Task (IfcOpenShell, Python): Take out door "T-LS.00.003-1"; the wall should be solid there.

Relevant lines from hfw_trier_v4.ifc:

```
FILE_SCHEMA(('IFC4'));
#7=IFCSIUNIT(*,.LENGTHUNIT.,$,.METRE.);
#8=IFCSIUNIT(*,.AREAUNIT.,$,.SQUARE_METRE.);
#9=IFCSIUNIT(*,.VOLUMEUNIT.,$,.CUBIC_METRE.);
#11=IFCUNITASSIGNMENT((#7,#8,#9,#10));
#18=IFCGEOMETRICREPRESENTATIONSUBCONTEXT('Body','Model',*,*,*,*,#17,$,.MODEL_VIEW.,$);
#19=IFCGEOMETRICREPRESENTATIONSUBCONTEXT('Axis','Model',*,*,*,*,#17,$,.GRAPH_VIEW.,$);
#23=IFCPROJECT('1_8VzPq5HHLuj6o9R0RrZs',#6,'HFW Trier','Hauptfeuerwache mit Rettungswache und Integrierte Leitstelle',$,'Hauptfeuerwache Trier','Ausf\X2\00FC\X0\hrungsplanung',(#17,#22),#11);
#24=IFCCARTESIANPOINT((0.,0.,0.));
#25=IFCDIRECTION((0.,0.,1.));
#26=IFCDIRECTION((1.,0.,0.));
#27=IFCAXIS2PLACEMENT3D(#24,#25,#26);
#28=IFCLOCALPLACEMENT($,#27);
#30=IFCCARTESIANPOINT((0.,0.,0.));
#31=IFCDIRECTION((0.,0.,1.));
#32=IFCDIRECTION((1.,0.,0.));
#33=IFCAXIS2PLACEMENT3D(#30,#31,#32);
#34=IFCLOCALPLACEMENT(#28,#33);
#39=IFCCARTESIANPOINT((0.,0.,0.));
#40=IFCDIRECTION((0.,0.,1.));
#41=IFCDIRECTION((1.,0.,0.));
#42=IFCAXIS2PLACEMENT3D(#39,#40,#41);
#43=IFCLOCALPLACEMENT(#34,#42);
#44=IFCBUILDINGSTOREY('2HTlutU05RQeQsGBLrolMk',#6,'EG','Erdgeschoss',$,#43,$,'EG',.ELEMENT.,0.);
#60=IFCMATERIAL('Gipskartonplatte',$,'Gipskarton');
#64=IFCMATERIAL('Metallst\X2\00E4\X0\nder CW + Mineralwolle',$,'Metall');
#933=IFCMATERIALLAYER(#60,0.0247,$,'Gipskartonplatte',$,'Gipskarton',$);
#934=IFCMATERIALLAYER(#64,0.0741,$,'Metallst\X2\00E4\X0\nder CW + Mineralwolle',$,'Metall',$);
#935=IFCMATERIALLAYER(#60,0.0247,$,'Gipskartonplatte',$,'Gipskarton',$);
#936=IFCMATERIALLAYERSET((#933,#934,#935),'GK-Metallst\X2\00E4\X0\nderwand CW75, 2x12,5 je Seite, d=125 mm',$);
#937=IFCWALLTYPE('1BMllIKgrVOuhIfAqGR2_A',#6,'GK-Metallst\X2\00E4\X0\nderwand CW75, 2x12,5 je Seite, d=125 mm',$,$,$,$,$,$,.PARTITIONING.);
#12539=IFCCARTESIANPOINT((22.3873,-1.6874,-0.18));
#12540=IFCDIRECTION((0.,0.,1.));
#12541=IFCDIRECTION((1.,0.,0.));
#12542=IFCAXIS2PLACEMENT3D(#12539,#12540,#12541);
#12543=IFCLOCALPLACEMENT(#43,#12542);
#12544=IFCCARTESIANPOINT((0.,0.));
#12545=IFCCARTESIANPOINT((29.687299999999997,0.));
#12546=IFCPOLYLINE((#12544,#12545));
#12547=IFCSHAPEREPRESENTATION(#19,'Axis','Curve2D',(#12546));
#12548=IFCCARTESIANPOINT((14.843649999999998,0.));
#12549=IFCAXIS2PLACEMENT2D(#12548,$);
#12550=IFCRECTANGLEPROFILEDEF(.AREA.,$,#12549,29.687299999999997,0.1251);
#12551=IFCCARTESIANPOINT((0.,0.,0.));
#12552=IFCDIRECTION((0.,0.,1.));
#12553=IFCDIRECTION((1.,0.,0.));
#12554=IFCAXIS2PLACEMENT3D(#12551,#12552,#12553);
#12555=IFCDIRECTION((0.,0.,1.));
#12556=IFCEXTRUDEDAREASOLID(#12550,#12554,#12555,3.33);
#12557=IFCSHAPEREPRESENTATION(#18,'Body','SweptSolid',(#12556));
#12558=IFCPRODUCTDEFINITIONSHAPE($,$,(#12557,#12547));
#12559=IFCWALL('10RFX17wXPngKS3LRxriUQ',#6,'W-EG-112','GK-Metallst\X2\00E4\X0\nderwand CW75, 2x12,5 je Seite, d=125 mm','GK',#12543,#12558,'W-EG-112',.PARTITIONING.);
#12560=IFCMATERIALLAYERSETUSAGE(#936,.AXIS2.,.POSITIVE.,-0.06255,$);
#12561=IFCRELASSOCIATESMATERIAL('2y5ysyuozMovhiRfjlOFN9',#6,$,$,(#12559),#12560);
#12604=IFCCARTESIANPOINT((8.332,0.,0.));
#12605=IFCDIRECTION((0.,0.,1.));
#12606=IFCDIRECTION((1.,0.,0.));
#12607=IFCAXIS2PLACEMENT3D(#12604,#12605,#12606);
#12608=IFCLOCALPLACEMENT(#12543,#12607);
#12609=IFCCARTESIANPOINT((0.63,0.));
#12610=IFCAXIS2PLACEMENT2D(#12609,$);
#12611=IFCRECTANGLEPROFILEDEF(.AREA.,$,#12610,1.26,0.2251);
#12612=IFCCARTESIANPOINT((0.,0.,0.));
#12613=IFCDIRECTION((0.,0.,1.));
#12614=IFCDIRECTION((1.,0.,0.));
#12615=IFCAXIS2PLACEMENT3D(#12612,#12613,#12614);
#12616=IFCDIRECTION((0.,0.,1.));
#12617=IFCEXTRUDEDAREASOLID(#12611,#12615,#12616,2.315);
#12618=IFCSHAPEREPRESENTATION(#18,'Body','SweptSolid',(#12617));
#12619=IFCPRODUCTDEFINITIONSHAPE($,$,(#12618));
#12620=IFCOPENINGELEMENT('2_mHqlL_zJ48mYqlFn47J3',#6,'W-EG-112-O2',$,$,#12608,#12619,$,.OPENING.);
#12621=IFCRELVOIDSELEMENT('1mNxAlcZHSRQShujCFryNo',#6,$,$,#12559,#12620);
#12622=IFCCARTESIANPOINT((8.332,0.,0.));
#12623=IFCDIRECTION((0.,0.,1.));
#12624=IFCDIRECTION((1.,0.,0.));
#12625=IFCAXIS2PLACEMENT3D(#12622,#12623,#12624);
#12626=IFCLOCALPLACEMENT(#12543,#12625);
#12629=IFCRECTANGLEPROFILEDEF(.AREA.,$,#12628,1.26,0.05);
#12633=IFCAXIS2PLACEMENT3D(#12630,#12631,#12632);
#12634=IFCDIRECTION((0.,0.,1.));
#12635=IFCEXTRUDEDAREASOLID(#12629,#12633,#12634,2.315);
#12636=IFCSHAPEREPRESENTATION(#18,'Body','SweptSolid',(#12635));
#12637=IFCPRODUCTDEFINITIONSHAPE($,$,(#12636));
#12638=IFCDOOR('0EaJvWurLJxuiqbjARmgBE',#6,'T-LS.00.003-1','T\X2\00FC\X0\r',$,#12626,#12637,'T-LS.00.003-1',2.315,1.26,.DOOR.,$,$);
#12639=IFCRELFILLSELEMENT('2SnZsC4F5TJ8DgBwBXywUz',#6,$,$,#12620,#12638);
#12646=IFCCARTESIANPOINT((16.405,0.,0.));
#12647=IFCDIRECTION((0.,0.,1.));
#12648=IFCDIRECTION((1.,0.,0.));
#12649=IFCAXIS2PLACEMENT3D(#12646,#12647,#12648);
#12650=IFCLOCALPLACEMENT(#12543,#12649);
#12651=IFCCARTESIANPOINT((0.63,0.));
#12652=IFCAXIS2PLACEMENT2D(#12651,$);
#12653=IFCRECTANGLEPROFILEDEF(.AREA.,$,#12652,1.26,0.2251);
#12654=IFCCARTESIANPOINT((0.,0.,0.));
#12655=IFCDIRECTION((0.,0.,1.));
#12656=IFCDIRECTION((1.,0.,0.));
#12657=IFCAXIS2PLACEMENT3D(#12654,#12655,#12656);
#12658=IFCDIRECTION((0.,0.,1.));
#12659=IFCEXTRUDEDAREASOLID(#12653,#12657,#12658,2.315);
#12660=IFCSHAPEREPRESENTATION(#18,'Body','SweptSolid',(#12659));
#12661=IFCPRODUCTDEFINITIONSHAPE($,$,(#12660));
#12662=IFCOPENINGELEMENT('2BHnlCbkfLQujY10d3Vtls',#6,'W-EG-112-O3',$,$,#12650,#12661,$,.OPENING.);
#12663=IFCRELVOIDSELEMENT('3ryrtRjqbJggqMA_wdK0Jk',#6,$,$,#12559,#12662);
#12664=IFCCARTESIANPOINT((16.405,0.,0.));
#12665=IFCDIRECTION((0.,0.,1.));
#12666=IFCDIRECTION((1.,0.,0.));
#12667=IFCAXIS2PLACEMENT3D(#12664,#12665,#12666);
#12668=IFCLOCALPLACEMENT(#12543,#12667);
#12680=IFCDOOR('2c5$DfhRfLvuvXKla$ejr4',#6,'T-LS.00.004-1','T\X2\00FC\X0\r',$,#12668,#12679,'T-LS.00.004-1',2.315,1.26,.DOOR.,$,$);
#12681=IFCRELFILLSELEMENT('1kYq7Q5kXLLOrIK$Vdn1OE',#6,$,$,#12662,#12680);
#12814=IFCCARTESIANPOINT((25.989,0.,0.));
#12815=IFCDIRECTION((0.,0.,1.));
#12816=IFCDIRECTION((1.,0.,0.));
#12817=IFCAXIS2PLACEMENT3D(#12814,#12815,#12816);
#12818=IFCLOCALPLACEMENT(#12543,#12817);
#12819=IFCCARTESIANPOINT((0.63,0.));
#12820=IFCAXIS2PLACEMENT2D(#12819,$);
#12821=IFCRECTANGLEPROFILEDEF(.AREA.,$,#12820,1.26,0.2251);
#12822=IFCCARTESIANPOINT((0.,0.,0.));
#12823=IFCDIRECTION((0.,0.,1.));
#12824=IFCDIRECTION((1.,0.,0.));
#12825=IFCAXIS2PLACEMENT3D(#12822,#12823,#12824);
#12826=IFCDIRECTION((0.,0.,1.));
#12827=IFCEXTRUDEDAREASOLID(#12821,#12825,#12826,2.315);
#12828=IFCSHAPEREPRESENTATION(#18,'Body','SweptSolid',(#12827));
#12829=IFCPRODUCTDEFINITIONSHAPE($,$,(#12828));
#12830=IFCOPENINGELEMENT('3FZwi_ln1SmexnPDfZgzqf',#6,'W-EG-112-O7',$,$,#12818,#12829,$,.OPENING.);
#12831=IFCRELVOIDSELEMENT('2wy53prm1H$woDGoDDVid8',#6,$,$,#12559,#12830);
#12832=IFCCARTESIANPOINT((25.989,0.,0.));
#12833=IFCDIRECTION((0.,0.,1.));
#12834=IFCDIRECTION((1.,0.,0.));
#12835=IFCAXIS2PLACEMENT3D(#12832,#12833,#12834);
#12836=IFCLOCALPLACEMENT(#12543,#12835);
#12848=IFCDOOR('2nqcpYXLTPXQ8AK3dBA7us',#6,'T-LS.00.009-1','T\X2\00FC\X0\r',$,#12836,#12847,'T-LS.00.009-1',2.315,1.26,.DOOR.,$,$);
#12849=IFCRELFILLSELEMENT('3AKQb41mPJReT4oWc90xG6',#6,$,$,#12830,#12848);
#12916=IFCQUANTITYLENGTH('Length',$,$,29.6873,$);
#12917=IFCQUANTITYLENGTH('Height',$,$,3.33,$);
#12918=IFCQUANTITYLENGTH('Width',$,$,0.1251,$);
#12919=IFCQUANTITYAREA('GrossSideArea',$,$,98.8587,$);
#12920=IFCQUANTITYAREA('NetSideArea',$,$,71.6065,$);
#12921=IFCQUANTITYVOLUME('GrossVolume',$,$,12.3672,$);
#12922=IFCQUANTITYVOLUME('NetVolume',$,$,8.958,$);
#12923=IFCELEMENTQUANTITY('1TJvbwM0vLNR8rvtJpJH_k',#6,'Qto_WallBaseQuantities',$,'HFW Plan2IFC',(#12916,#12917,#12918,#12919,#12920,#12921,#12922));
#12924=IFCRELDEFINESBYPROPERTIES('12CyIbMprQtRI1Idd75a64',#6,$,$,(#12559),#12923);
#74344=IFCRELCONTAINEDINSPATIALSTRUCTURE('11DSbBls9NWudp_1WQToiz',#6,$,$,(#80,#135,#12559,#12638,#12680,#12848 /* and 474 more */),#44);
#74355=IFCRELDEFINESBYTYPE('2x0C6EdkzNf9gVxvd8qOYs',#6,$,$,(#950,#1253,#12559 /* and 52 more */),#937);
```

```python
import ifcopenshell
import ifcopenshell.api.feature
import ifcopenshell.api.pset
import ifcopenshell.api.root
import ifcopenshell.geom
import ifcopenshell.util.element
import ifcopenshell.util.shape
import ifcopenshell.util.unit

model = ifcopenshell.open("hfw_trier_v4.ifc")
area_scale = ifcopenshell.util.unit.calculate_unit_scale(model, "AREAUNIT")
volume_scale = ifcopenshell.util.unit.calculate_unit_scale(model, "VOLUMEUNIT")
settings = ifcopenshell.geom.settings()


def volume(element):
    """Net volume in cubic metres, openings subtracted."""
    shape = ifcopenshell.geom.create_shape(settings, element)
    return ifcopenshell.util.shape.get_volume(shape.geometry)


door = model.by_guid("0EaJvWurLJxuiqbjARmgBE")
opening = door.FillsVoids[0].RelatingOpeningElement
wall = opening.VoidsElements[0].RelatingBuildingElement
before = volume(wall)

ifcopenshell.api.root.remove_product(model, product=door)
ifcopenshell.api.feature.remove_feature(model, feature=opening)

after = volume(wall)
thickness = 0.1251  # wall thickness in metres

# Update the wall's stored quantities.
qto = model.by_id(ifcopenshell.util.element.get_pset(wall, "Qto_WallBaseQuantities", should_inherit=False)["id"])
ifcopenshell.api.pset.edit_qto(model, qto=qto, properties={
    "NetSideArea": after / thickness / area_scale,
    "NetVolume": after / volume_scale,
})

print(f"wall volume {before:.3f} -> {after:.3f} m3")

model.write("hfw_trier_v4_v2.ifc")
```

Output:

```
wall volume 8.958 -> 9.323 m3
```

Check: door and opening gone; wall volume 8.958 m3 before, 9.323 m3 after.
